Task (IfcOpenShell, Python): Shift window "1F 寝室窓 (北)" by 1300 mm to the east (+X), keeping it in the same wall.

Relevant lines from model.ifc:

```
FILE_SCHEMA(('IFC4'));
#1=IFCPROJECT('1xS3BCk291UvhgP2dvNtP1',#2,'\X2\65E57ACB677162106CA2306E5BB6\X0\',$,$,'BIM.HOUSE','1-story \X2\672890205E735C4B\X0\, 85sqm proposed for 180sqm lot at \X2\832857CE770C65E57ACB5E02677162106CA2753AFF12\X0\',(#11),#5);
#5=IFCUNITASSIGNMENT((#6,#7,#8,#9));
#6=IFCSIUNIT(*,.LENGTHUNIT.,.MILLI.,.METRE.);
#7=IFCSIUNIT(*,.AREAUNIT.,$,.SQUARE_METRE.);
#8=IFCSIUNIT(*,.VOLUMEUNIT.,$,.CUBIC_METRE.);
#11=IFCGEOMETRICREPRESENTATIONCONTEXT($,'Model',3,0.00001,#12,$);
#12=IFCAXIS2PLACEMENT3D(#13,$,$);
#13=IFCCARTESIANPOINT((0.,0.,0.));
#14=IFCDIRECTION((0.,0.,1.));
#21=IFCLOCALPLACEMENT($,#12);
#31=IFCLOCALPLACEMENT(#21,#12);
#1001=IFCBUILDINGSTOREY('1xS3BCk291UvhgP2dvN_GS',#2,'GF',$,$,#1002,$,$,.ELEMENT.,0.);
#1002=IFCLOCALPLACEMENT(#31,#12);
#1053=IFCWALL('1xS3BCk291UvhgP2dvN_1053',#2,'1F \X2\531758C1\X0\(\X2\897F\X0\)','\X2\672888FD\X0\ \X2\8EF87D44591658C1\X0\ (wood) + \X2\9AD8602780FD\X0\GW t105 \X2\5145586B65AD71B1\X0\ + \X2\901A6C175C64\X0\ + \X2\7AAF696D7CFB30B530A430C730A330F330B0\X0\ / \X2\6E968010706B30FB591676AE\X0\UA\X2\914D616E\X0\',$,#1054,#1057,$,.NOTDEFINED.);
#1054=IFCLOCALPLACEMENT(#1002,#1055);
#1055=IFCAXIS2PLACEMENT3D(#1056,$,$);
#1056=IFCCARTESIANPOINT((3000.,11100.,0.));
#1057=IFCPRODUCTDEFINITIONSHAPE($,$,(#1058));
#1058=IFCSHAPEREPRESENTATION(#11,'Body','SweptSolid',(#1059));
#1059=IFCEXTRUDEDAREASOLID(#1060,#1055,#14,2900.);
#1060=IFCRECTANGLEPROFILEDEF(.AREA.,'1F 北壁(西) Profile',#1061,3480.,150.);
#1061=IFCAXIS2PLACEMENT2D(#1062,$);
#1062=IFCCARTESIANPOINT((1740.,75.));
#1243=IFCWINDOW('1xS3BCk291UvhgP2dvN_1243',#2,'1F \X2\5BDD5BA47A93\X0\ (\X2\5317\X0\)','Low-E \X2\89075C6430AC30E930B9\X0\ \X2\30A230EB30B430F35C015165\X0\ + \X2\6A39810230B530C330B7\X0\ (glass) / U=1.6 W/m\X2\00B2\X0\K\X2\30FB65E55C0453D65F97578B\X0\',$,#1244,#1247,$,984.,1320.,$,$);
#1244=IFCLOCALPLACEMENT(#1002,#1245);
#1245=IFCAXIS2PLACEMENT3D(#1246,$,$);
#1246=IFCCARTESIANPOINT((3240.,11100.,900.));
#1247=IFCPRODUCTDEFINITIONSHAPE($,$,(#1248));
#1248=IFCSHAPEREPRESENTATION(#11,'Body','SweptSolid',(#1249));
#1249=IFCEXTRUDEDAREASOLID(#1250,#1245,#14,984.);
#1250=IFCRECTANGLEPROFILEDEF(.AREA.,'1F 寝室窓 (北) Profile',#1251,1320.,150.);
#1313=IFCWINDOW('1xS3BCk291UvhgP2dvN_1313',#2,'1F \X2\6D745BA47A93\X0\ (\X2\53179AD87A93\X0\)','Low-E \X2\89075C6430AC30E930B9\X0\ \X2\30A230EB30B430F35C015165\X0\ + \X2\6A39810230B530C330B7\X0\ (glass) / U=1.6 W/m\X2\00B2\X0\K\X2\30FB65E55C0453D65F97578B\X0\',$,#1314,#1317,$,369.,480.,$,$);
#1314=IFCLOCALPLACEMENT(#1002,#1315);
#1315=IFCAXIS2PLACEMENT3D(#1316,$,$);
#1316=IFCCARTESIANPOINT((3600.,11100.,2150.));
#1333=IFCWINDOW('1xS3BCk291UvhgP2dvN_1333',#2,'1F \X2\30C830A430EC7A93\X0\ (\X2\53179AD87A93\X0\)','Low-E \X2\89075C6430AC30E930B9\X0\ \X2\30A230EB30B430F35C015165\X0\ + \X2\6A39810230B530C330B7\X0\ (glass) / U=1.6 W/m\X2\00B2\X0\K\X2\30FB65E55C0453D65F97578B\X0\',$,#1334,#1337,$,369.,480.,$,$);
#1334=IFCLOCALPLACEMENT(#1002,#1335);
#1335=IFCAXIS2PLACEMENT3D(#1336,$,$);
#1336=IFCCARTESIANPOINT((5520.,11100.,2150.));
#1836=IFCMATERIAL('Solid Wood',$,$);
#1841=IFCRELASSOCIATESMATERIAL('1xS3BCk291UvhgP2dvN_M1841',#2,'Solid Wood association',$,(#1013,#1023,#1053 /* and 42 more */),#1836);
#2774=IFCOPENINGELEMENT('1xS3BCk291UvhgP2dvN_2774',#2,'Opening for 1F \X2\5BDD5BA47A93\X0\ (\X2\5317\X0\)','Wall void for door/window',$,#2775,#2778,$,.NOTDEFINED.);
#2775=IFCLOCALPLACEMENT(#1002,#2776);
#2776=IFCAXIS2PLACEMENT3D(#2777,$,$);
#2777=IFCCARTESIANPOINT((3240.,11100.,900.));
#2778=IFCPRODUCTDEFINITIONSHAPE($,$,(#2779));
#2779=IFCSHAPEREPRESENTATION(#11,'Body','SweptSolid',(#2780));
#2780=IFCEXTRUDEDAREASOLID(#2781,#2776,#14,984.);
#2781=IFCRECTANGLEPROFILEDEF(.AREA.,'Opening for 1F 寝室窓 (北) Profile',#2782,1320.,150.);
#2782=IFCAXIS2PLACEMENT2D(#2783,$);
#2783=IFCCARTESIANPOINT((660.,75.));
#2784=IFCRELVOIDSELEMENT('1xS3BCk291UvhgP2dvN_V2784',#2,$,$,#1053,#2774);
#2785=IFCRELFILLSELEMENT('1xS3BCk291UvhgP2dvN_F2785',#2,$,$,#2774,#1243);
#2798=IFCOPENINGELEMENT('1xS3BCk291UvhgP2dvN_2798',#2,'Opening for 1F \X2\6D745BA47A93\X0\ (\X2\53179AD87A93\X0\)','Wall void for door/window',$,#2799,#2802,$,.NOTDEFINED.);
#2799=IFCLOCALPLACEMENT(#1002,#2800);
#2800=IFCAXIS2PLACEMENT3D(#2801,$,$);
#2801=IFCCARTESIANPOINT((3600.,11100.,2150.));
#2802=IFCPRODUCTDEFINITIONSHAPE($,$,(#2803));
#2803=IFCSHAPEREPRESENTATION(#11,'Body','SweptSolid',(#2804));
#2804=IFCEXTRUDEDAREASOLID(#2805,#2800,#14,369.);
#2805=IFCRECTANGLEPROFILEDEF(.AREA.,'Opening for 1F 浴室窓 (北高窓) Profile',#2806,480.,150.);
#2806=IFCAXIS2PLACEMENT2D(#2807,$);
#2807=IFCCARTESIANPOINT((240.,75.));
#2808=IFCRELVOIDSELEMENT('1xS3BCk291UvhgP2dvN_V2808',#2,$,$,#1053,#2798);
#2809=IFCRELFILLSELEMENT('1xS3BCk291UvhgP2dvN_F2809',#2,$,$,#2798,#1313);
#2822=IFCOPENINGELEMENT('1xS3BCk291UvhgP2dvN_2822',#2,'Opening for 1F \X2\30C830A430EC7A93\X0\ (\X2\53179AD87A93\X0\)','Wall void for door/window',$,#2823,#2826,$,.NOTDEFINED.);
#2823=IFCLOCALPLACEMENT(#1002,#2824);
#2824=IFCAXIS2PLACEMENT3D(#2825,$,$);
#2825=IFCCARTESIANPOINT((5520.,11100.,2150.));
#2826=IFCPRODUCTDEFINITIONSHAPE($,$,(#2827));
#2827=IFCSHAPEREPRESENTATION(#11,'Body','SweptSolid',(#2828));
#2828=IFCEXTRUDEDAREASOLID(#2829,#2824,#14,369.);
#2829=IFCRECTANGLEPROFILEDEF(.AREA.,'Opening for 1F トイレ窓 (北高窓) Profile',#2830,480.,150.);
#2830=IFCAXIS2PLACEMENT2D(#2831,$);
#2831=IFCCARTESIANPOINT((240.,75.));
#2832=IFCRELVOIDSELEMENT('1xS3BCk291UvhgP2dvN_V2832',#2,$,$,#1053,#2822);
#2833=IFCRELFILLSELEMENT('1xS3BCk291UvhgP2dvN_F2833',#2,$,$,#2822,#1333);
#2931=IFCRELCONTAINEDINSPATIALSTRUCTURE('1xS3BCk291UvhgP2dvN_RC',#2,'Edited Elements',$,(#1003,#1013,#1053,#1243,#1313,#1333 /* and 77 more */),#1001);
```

```python
import ifcopenshell
import ifcopenshell.api.geometry
import ifcopenshell.util.placement
import ifcopenshell.util.unit

model = ifcopenshell.open("model.ifc")
unit_scale = ifcopenshell.util.unit.calculate_unit_scale(model)

window = model.by_guid("1xS3BCk291UvhgP2dvN_1243")
opening = window.FillsVoids[0].RelatingOpeningElement
wall = opening.VoidsElements[0].RelatingBuildingElement

wall_matrix = ifcopenshell.util.placement.get_local_placement(wall.ObjectPlacement)
shift = wall_matrix[:3, 0] * 1.3 / unit_scale
before = ifcopenshell.util.placement.get_local_placement(window.ObjectPlacement)[:3, 3].copy()

# The window is not placed relative to its opening, so move both.
for product in (opening, window):
    matrix = ifcopenshell.util.placement.get_local_placement(product.ObjectPlacement)
    matrix[:3, 3] += shift
    ifcopenshell.api.geometry.edit_object_placement(model, product=product, matrix=matrix, is_si=False)

after = ifcopenshell.util.placement.get_local_placement(window.ObjectPlacement)[:3, 3]
print("window moved by", (after - before).round(3) + 0.0)

model.write("model_v2.ifc")
```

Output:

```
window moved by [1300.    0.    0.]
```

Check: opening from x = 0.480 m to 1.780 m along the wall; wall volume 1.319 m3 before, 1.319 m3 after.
